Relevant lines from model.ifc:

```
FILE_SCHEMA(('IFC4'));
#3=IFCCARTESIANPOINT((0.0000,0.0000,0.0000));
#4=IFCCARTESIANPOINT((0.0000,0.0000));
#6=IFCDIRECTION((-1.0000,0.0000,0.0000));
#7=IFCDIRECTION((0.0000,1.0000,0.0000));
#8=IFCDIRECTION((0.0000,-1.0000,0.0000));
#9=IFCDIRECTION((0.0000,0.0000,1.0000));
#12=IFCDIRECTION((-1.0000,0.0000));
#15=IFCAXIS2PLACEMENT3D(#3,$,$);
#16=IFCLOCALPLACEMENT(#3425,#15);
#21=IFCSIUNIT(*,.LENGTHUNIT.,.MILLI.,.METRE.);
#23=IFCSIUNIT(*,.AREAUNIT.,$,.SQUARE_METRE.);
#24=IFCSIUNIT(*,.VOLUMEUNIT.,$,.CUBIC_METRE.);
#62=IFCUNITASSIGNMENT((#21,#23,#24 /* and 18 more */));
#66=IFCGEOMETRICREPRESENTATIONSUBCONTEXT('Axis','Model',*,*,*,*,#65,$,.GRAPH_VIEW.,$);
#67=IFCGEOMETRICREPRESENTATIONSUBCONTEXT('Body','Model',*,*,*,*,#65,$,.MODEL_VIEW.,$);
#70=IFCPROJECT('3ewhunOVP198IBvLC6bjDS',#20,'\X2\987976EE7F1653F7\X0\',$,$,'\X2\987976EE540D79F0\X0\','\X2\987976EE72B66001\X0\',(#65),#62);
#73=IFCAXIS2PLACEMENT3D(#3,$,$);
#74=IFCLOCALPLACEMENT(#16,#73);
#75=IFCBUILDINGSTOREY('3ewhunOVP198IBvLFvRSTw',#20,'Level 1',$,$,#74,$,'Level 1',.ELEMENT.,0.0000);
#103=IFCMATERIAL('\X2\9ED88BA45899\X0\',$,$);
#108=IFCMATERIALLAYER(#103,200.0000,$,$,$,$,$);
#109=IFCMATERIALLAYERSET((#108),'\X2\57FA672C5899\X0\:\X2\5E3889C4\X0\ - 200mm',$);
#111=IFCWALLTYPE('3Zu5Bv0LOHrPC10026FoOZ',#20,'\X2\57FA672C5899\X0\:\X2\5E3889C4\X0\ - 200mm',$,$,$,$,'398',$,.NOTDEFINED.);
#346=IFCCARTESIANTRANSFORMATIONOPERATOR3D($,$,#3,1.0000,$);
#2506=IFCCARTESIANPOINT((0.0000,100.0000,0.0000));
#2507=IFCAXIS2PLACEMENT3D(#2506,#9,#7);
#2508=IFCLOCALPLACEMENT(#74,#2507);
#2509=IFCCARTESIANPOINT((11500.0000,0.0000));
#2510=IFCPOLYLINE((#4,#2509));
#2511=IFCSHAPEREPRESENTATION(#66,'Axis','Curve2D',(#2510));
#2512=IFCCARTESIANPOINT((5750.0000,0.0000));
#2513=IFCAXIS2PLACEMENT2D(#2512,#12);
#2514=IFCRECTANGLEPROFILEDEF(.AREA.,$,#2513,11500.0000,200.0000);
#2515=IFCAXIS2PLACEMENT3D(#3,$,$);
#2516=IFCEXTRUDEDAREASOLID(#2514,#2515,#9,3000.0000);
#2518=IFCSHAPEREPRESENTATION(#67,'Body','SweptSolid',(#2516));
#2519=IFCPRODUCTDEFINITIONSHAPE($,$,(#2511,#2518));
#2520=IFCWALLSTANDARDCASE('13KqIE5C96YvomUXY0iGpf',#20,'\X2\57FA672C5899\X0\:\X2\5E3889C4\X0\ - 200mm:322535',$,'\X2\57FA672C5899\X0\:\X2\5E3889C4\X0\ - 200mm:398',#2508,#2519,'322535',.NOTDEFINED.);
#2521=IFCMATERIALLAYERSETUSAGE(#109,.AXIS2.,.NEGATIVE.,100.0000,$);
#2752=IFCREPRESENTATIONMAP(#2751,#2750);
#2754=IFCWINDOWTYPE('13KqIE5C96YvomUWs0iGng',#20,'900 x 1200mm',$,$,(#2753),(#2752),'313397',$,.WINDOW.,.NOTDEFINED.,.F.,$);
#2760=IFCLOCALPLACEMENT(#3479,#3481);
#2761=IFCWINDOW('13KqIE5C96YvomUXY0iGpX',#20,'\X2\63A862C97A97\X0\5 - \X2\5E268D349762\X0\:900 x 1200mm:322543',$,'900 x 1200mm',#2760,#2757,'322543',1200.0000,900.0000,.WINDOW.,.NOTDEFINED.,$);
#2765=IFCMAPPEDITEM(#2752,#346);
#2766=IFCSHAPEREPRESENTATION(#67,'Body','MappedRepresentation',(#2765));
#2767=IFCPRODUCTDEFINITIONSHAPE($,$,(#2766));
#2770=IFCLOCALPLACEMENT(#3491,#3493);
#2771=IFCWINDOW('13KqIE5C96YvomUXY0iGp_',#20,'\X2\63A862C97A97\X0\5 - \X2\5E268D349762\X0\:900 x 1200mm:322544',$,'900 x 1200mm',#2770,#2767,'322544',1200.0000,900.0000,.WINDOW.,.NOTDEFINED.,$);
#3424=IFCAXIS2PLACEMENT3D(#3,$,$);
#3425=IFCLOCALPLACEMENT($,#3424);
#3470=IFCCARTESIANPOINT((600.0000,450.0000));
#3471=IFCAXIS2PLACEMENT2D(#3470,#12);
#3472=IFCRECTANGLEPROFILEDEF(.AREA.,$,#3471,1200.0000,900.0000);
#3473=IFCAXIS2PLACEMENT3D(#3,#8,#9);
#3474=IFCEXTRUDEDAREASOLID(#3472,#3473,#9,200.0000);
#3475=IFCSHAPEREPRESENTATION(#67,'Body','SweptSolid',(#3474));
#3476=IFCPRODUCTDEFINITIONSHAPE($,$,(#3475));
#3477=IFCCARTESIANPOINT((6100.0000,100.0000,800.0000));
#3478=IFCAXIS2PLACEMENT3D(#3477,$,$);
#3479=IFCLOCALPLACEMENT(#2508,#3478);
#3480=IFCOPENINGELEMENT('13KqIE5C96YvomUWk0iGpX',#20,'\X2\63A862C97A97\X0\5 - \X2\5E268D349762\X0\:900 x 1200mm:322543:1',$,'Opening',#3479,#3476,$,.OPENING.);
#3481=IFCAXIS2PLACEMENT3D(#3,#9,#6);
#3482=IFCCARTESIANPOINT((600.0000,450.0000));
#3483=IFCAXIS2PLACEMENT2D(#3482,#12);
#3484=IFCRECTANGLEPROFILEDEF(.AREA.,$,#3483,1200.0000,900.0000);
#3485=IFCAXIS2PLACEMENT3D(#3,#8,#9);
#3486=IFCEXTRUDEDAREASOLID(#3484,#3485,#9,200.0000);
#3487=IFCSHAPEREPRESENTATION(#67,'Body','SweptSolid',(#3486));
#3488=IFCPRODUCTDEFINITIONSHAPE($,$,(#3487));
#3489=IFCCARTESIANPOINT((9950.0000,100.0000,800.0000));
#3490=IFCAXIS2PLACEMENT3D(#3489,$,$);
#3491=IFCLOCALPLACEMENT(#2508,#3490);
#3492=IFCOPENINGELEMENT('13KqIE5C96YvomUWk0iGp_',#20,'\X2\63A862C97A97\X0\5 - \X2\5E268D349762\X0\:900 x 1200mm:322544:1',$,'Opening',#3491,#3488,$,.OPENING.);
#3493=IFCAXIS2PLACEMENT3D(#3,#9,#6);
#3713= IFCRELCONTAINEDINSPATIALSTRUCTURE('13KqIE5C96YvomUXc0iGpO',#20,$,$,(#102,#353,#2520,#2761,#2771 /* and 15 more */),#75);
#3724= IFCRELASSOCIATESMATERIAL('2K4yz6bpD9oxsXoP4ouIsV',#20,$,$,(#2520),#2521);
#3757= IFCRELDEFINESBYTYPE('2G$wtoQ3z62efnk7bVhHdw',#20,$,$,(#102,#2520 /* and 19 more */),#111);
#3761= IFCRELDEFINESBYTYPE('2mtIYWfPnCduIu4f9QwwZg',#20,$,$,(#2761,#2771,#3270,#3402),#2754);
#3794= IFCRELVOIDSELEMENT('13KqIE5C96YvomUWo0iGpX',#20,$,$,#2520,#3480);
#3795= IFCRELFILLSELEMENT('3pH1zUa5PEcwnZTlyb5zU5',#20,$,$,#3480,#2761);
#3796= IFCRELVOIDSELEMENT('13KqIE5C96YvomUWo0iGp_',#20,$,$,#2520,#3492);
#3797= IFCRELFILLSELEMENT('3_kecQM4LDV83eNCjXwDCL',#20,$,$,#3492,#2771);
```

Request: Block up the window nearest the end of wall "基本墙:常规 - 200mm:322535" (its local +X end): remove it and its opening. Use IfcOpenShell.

```python
import ifcopenshell
import ifcopenshell.api.feature
import ifcopenshell.api.root
import ifcopenshell.geom
import ifcopenshell.util.shape

model = ifcopenshell.open("model.ifc")
settings = ifcopenshell.geom.settings()


def volume(element):
    """Net volume in cubic metres, openings subtracted."""
    shape = ifcopenshell.geom.create_shape(settings, element)
    return ifcopenshell.util.shape.get_volume(shape.geometry)


window = model.by_guid("13KqIE5C96YvomUXY0iGp_")
opening = window.FillsVoids[0].RelatingOpeningElement
wall = opening.VoidsElements[0].RelatingBuildingElement
before = volume(wall)

ifcopenshell.api.root.remove_product(model, product=window)
ifcopenshell.api.feature.remove_feature(model, feature=opening)

after = volume(wall)

print(f"wall volume {before:.3f} -> {after:.3f} m3")

model.write("model_v2.ifc")
```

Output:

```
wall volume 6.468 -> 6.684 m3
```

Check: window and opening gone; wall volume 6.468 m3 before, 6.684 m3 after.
